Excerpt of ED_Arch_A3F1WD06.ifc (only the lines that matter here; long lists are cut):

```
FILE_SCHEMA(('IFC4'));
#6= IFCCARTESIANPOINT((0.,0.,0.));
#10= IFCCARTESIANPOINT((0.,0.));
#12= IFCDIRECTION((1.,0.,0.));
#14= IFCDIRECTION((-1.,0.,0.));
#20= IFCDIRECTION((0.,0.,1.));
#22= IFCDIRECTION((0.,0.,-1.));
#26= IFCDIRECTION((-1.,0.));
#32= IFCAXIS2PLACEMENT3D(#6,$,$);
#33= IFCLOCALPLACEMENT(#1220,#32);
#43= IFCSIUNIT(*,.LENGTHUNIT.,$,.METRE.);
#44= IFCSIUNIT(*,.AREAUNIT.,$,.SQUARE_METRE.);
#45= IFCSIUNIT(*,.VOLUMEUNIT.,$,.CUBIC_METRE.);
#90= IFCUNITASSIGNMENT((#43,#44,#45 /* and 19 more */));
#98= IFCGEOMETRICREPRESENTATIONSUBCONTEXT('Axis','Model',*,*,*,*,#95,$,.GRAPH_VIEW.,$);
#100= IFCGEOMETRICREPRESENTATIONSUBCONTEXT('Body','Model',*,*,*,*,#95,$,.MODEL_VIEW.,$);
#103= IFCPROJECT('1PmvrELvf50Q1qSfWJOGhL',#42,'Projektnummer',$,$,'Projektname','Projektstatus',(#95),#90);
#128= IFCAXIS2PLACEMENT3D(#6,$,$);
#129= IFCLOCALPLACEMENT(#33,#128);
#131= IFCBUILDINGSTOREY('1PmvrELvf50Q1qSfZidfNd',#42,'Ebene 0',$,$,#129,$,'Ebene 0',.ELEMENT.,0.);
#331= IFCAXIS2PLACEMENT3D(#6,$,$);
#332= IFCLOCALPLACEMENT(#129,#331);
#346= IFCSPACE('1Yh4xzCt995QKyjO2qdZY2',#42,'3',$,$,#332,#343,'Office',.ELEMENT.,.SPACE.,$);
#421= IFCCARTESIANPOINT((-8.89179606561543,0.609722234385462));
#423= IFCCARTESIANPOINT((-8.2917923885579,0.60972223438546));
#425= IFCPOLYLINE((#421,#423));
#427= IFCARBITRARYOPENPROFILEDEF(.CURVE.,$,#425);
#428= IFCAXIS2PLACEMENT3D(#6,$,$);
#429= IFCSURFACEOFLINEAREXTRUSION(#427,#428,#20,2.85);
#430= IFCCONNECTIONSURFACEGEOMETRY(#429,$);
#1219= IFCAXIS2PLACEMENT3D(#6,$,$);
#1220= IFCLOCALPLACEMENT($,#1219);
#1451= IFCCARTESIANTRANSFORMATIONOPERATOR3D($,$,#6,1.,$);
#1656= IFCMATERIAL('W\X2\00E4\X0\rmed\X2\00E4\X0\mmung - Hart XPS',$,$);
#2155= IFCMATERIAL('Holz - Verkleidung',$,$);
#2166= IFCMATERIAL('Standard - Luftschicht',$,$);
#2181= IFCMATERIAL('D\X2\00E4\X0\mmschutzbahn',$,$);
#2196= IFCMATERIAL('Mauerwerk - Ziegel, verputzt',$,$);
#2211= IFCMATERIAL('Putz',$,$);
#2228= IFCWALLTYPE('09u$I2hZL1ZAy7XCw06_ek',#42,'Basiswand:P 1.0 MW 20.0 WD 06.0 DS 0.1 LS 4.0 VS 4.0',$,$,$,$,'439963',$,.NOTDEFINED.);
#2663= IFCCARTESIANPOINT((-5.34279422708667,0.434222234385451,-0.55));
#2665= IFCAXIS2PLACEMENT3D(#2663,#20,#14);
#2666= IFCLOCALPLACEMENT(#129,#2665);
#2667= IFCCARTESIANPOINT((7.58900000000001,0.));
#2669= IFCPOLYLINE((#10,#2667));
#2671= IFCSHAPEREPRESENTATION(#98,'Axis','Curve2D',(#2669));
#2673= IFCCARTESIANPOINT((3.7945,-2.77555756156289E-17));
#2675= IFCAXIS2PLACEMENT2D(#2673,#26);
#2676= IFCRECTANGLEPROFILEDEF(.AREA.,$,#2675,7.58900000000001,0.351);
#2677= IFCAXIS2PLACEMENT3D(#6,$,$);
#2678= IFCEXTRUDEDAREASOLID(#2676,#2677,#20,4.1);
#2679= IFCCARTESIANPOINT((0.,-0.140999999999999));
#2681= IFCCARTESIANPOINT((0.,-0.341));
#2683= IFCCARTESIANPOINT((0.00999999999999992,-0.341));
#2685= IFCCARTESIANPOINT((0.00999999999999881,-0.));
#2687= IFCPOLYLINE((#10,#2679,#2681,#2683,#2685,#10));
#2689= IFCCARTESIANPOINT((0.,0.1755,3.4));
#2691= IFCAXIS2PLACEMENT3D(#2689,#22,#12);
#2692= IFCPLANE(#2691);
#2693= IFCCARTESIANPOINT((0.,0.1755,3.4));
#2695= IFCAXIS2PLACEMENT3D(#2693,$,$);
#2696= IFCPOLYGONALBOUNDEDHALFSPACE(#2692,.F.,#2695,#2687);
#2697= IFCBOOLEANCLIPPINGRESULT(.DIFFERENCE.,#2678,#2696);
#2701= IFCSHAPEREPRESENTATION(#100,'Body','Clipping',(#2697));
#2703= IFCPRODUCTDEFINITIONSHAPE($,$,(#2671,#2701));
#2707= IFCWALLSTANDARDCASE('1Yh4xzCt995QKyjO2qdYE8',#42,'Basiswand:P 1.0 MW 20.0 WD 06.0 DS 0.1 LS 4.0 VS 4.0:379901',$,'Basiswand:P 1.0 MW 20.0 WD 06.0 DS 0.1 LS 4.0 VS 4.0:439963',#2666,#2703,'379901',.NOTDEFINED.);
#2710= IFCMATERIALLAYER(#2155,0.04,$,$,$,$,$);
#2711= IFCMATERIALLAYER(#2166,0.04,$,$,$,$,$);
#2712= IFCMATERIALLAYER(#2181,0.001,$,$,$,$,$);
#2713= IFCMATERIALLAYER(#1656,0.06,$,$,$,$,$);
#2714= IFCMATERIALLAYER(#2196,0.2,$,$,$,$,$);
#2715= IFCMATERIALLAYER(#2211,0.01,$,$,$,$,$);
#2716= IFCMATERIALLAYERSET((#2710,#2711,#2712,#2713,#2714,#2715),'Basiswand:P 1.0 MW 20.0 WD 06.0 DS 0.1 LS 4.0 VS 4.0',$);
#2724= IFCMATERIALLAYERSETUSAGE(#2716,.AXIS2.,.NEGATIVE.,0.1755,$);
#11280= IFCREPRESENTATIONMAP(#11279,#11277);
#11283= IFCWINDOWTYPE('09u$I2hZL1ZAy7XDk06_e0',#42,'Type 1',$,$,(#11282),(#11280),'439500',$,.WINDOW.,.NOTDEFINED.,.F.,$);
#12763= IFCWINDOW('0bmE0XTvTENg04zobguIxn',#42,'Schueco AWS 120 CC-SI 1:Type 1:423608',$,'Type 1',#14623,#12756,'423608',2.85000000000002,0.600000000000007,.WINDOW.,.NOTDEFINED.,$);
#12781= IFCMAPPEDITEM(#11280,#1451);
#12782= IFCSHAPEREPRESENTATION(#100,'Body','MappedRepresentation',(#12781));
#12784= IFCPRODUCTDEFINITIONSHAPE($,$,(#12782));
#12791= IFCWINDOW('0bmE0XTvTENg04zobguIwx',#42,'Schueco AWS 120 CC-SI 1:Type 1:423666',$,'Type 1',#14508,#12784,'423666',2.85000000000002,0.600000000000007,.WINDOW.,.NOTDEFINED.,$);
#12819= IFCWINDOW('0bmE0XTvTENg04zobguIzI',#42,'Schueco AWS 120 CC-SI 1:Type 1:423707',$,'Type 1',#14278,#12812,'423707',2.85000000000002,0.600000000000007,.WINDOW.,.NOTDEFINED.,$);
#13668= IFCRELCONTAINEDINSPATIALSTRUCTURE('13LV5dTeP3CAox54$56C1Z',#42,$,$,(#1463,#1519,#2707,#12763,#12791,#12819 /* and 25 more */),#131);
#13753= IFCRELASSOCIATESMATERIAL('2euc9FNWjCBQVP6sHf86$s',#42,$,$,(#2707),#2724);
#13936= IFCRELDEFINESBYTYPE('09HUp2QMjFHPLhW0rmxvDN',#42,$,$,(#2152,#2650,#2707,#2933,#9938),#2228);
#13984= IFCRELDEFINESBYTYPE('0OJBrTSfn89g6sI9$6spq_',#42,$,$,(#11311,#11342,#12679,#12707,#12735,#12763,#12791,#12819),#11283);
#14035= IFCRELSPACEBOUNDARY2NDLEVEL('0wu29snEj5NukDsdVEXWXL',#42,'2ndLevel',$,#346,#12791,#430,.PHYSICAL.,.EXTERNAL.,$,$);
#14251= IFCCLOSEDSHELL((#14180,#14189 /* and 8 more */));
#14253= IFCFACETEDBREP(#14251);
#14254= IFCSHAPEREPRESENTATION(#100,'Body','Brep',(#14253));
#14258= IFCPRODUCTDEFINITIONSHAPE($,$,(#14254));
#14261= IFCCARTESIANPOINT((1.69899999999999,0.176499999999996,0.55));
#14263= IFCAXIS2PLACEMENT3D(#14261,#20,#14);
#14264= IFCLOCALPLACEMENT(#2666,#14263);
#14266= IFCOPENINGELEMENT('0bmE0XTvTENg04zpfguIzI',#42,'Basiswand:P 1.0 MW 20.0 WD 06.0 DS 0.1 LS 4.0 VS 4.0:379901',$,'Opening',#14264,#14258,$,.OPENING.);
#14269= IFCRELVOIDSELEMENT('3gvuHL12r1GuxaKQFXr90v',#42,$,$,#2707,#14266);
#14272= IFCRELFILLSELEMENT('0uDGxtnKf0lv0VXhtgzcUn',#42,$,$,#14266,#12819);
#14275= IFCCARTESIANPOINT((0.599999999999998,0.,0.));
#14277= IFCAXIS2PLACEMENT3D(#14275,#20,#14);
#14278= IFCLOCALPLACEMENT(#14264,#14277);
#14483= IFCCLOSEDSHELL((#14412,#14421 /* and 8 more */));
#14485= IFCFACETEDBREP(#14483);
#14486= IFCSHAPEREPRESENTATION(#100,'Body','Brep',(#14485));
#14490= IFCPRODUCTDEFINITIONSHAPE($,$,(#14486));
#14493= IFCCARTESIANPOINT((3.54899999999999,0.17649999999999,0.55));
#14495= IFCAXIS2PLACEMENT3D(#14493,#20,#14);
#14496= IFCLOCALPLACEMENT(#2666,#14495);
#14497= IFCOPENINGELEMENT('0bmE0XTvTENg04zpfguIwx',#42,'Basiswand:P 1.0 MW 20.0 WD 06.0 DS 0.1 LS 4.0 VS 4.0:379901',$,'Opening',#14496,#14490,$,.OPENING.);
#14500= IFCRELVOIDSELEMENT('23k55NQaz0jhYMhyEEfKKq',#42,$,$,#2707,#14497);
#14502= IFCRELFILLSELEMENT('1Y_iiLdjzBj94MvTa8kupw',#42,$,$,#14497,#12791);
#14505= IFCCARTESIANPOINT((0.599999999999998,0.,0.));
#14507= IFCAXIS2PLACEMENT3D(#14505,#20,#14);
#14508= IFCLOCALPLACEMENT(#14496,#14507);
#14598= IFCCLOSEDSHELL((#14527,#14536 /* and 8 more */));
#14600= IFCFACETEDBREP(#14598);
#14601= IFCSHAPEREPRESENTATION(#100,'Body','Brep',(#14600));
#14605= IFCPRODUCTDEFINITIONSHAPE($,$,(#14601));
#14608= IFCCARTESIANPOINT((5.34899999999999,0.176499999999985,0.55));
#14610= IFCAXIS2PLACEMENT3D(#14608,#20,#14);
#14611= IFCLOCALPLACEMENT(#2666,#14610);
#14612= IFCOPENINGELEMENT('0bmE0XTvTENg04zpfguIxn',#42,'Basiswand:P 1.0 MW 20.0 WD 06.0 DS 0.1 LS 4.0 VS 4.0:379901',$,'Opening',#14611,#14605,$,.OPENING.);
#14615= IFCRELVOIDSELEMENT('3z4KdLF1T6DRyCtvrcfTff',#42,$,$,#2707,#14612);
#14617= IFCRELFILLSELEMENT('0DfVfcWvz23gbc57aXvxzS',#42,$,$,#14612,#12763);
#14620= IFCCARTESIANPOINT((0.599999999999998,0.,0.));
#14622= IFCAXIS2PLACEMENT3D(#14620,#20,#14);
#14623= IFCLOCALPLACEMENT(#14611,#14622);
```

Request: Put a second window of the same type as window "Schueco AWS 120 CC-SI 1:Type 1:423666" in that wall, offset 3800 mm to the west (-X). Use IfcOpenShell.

```python
import numpy as np
import ifcopenshell
import ifcopenshell.api.feature
import ifcopenshell.api.geometry
import ifcopenshell.api.root
import ifcopenshell.geom
import ifcopenshell.util.element
import ifcopenshell.util.placement
import ifcopenshell.util.shape

model = ifcopenshell.open("ED_Arch_A3F1WD06.ifc")
settings = ifcopenshell.geom.settings()


def volume(element):
    """Net volume in cubic metres, openings subtracted."""
    shape = ifcopenshell.geom.create_shape(settings, element)
    return ifcopenshell.util.shape.get_volume(shape.geometry)


def reuse_history(source, copy):
    """copy_class also copies each property set's owner history, people and application; keep the originals."""
    for rel in copy.IsDefinedBy:
        if rel.is_a("IfcRelDefinesByProperties") and (history := rel.RelatingPropertyDefinition.OwnerHistory):
            rel.RelatingPropertyDefinition.OwnerHistory = source.OwnerHistory
            ifcopenshell.util.element.remove_deep2(model, history)


window = model.by_guid("0bmE0XTvTENg04zobguIwx")
opening = window.FillsVoids[0].RelatingOpeningElement
wall = opening.VoidsElements[0].RelatingBuildingElement
before = volume(wall)
shift = ifcopenshell.util.placement.get_local_placement(wall.ObjectPlacement)[:3, 0] * 3.8

# copy_class copies the void relationship, type, container and properties, but no geometry.
new_opening = ifcopenshell.api.root.copy_class(model, product=opening)
new_opening.Representation = ifcopenshell.util.element.copy_deep(
    model, opening.Representation, exclude=["IfcGeometricRepresentationContext", "IfcRepresentationMap"]
)
new_opening.Name = "Basiswand:P 1.0 MW 20.0 WD 06.0 DS 0.1 LS 4.0 VS 4.0"
new_window = ifcopenshell.api.root.copy_class(model, product=window)
new_window.Representation = ifcopenshell.util.element.copy_deep(
    model, window.Representation, exclude=["IfcGeometricRepresentationContext", "IfcRepresentationMap"]
)
new_window.Name = "Schueco AWS 120 CC-SI 1:Type 1"
new_window.Tag = None
reuse_history(window, new_window)
ifcopenshell.api.feature.add_filling(model, opening=new_opening, element=new_window)

for old, new in ((opening, new_opening), (window, new_window)):
    matrix = ifcopenshell.util.placement.get_local_placement(old.ObjectPlacement)
    matrix[:3, 3] += shift
    ifcopenshell.api.geometry.edit_object_placement(model, product=new, matrix=matrix, is_si=False)

# The copied space boundaries still share their surfaces with the original.
for rel in new_window.ProvidesBoundaries:
    if rel.ConnectionGeometry:
        rel.ConnectionGeometry = ifcopenshell.util.element.copy_deep(model, rel.ConnectionGeometry)

# Space boundary surfaces are stored in each space's coordinates; move them too.
for rel in new_window.ProvidesBoundaries:
    if not rel.ConnectionGeometry:
        continue
    surface = rel.ConnectionGeometry.SurfaceOnRelatingElement
    space_matrix = ifcopenshell.util.placement.get_local_placement(rel.RelatingSpace.ObjectPlacement)
    point = np.array(surface.Position.Location.Coordinates) + space_matrix[:3, :3].T @ shift
    surface.Position = model.createIfcAxis2Placement3D(
        model.createIfcCartesianPoint(point.tolist()), surface.Position.Axis, surface.Position.RefDirection
    )

after = volume(wall)

print(f"wall volume {before:.3f} -> {after:.3f} m3")

model.write("ED_Arch_A3F1WD06_edited.ifc")
```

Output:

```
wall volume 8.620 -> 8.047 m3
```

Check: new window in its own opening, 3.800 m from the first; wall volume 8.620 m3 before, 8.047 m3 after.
